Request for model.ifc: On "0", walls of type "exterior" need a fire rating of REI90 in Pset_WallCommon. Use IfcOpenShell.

First a look at what the model holds.

```python
import ifcopenshell
import ifcopenshell.util.element

model = ifcopenshell.open("model.ifc")
print(model.schema)
storey = next(s for s in model.by_type("IfcBuildingStorey") if s.Name == "0")
walls = [e for e in ifcopenshell.util.element.get_decomposition(storey) if e.is_a("IfcWall")]
seen = {}
for e in walls:
    element_type = ifcopenshell.util.element.get_type(e)
    key = (element_type.Name if element_type != e and element_type else None, ifcopenshell.util.element.get_pset(e, "Pset_WallCommon", "FireRating"))
    seen[key] = seen.get(key, 0) + 1
for (name, value), count in sorted(seen.items(), key=str):
    print(count, "x", name, "|", value)
```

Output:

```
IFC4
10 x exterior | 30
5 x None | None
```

```python
import ifcopenshell
import ifcopenshell.api.pset
import ifcopenshell.util.element

model = ifcopenshell.open("model.ifc")

storey = next(s for s in model.by_type("IfcBuildingStorey") if s.Name == "0")
walls = [e for e in ifcopenshell.util.element.get_decomposition(storey) if e.is_a("IfcWall")]

count = 0
for e in walls:
    element_type = ifcopenshell.util.element.get_type(e)
    if element_type in (None, e) or element_type.Name != "exterior":
        continue
    # add_pset returns the element's existing set when there is one.
    pset = ifcopenshell.api.pset.add_pset(model, product=e, name="Pset_WallCommon")
    ifcopenshell.api.pset.edit_pset(model, pset=pset, properties={"FireRating": "REI90"})
    count += 1

print(count, "walls updated")

model.write("model_rev.ifc")
```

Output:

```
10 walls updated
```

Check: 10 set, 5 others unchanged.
